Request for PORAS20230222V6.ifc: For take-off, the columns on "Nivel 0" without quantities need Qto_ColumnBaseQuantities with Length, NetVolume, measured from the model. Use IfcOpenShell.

First a look at what the model holds.

```python
import ifcopenshell
import ifcopenshell.util.element
import ifcopenshell.util.unit

model = ifcopenshell.open("PORAS20230222V6.ifc")
print(model.schema)
for unit_type in ("LENGTHUNIT", "AREAUNIT", "VOLUMEUNIT"):
    print(unit_type, ifcopenshell.util.unit.calculate_unit_scale(model, unit_type))
storey = next(s for s in model.by_type("IfcBuildingStorey") if s.Name == "Nivel 0")
columns = [e for e in ifcopenshell.util.element.get_decomposition(storey) if e.is_a("IfcColumn")]
for e in sorted(columns, key=lambda e: e.id()):
    print(e.id(), e.is_a(), e.Name, list(ifcopenshell.util.element.get_psets(e, qtos_only=True)), sep=" | ")
```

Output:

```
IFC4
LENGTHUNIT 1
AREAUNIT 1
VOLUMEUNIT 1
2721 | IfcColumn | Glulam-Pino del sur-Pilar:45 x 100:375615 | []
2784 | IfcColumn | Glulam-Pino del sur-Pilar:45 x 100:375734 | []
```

```python
import ifcopenshell
import ifcopenshell.api.pset
import ifcopenshell.geom
import ifcopenshell.util.element
import ifcopenshell.util.shape
import ifcopenshell.util.unit

model = ifcopenshell.open("PORAS20230222V6.ifc")
unit_scale = ifcopenshell.util.unit.calculate_unit_scale(model)
volume_scale = ifcopenshell.util.unit.calculate_unit_scale(model, "VOLUMEUNIT")
settings = ifcopenshell.geom.settings()

storey = next(s for s in model.by_type("IfcBuildingStorey") if s.Name == "Nivel 0")
columns = [e for e in ifcopenshell.util.element.get_decomposition(storey) if e.is_a("IfcColumn")]

for e in sorted(columns, key=lambda e: e.id()):
    if ifcopenshell.util.element.get_psets(e, qtos_only=True, should_inherit=False):
        continue
    # Geometry comes back in metres, in the element's own axes.
    shape = ifcopenshell.geom.create_shape(settings, e)
    values = {
        "Length": ifcopenshell.util.shape.get_z(shape.geometry) / unit_scale,
        "NetVolume": ifcopenshell.util.shape.get_volume(shape.geometry) / volume_scale,
    }
    qto = ifcopenshell.api.pset.add_qto(model, product=e, name="Qto_ColumnBaseQuantities")
    ifcopenshell.api.pset.edit_qto(model, qto=qto, properties=values)
    print(e.id(), {k: round(v, 3) for k, v in values.items()})

model.write("PORAS20230222V6_rev.ifc")
```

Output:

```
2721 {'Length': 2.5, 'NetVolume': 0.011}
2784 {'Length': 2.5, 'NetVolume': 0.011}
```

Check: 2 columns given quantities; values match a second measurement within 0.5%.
